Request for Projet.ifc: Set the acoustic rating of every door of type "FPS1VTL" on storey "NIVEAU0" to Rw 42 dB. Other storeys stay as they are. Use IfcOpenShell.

First a look at what the model holds.

```python
import ifcopenshell
import ifcopenshell.util.element

model = ifcopenshell.open("Projet.ifc")
print(model.schema)
storey = next(s for s in model.by_type("IfcBuildingStorey") if s.Name == "NIVEAU0")
doors = [e for e in ifcopenshell.util.element.get_decomposition(storey) if e.is_a("IfcDoor")]
seen = {}
for e in doors:
    element_type = ifcopenshell.util.element.get_type(e)
    key = (element_type.Name if element_type != e and element_type else None, ifcopenshell.util.element.get_pset(e, "Pset_DoorCommon", "AcousticRating"))
    seen[key] = seen.get(key, 0) + 1
for (name, value), count in sorted(seen.items(), key=str):
    print(count, "x", name, "|", value)
```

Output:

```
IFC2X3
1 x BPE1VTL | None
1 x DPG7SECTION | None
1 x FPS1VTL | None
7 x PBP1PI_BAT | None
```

```python
import ifcopenshell
import ifcopenshell.api.pset
import ifcopenshell.util.element

model = ifcopenshell.open("Projet.ifc")

storey = next(s for s in model.by_type("IfcBuildingStorey") if s.Name == "NIVEAU0")
doors = [e for e in ifcopenshell.util.element.get_decomposition(storey) if e.is_a("IfcDoor")]

count = 0
for e in doors:
    element_type = ifcopenshell.util.element.get_type(e)
    if element_type in (None, e) or element_type.Name != "FPS1VTL":
        continue
    # add_pset returns the element's existing set when there is one.
    pset = ifcopenshell.api.pset.add_pset(model, product=e, name="Pset_DoorCommon")
    ifcopenshell.api.pset.edit_pset(model, pset=pset, properties={"AcousticRating": "Rw 42 dB"})
    count += 1

print(count, "doors updated")

model.write("Projet-out.ifc")
```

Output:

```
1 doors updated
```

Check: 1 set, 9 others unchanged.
